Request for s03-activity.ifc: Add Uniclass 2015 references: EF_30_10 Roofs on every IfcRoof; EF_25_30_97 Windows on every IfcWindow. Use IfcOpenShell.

First a look at what the model holds.

```python
import ifcopenshell

model = ifcopenshell.open("s03-activity.ifc")
print(model.schema)
print("classifications:", [c.Name for c in model.by_type("IfcClassification")])
for ifc_class in ("IfcDoor", "IfcRoof", "IfcStair", "IfcWall", "IfcWindow"):
    print(ifc_class, len(model.by_type(ifc_class)))
```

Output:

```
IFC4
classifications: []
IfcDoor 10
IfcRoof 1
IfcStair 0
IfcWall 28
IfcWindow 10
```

```python
import ifcopenshell
import ifcopenshell.api.classification

model = ifcopenshell.open("s03-activity.ifc")

system = ifcopenshell.api.classification.add_classification(model, classification="Uniclass 2015")

codes = {
    "IfcRoof": ("EF_30_10", "Roofs"),
    "IfcWindow": ("EF_25_30_97", "Windows"),
}
for ifc_class, (code, name) in codes.items():
    products = model.by_type(ifc_class)
    ifcopenshell.api.classification.add_reference(
        model, products=products, classification=system, identification=code, name=name
    )
    print(code, len(products))

model.write("s03-activity_updated.ifc")
```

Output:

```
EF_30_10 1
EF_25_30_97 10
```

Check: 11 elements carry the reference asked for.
